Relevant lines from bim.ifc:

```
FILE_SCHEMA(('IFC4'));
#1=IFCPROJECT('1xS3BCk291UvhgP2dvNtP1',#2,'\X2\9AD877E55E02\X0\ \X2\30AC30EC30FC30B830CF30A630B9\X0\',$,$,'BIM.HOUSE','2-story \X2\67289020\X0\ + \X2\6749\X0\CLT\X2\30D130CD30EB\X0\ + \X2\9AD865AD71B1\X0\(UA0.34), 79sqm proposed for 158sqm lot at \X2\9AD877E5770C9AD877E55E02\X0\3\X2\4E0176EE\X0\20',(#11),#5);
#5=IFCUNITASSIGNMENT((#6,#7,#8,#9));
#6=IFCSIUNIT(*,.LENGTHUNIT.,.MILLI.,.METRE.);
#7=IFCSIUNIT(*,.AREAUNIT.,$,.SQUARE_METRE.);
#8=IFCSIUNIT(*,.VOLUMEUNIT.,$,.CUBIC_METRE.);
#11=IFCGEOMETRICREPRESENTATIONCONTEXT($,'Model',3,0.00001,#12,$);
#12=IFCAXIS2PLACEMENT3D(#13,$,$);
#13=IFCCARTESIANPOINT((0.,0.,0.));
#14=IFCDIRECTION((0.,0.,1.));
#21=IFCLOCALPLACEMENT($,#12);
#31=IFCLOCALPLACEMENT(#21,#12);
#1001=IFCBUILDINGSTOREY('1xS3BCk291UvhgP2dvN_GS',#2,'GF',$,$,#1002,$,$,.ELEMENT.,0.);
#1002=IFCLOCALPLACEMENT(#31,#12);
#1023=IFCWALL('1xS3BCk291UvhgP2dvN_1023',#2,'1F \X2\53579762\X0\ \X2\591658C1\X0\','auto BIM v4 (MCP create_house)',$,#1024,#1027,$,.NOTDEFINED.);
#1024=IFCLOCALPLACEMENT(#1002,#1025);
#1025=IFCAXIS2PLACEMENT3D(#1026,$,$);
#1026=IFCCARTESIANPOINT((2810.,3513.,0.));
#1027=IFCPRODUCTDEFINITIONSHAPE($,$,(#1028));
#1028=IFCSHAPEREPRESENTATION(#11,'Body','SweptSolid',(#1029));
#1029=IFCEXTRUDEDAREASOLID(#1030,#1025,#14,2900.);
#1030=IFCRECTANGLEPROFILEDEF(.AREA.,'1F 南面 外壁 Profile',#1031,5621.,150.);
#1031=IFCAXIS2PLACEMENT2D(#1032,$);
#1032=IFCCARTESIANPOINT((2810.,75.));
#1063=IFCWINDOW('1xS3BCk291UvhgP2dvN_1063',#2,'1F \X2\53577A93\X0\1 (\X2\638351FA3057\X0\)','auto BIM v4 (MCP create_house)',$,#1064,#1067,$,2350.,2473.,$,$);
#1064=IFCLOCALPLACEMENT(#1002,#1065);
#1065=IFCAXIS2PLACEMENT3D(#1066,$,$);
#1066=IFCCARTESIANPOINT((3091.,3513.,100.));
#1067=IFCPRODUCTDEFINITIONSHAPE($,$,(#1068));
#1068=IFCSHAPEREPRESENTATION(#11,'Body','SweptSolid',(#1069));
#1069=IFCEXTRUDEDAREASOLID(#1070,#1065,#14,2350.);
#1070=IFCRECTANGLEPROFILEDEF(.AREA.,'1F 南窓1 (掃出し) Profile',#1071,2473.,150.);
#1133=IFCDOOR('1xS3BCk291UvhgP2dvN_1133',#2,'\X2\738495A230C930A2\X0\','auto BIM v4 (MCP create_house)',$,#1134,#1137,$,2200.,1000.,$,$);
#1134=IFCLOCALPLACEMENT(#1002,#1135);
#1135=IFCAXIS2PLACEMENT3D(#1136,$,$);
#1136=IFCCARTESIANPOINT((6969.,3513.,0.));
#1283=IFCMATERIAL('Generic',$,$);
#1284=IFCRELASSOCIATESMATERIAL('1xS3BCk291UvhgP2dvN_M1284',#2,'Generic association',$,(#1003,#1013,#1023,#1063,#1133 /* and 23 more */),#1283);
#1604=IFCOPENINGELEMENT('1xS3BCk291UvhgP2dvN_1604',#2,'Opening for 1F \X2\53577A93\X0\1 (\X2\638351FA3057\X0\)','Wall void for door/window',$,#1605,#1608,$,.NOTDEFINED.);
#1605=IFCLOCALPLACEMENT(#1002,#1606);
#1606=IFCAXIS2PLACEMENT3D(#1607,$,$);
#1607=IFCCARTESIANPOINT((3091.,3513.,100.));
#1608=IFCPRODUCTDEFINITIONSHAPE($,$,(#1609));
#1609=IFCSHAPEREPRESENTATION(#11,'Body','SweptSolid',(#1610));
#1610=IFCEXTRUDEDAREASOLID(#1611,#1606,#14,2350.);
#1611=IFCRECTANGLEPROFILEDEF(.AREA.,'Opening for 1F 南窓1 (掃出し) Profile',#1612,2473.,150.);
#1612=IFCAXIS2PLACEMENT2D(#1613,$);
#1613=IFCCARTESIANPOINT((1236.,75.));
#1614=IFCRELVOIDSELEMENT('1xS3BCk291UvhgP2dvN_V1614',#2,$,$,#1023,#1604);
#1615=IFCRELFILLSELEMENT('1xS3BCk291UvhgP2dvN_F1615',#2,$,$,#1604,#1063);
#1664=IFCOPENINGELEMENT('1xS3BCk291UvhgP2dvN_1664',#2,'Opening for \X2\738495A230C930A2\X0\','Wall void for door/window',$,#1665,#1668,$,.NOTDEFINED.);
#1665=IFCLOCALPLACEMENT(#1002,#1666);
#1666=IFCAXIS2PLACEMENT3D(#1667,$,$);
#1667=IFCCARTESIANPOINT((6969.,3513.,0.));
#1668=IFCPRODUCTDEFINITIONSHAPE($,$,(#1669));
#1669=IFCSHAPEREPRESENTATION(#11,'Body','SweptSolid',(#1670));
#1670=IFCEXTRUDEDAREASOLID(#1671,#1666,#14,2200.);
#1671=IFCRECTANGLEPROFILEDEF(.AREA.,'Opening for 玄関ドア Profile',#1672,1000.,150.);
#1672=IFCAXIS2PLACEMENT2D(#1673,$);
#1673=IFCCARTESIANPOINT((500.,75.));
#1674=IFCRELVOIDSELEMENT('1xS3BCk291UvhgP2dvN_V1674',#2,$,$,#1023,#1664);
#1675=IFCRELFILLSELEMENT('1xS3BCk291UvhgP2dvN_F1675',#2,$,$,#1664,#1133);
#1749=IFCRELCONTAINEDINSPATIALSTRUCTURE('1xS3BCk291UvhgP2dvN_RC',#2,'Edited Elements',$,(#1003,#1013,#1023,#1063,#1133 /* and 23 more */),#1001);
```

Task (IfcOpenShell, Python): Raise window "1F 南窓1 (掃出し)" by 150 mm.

```python
import numpy as np
import ifcopenshell
import ifcopenshell.api.geometry
import ifcopenshell.util.placement
import ifcopenshell.util.unit

model = ifcopenshell.open("bim.ifc")
unit_scale = ifcopenshell.util.unit.calculate_unit_scale(model)

window = model.by_guid("1xS3BCk291UvhgP2dvN_1063")
opening = window.FillsVoids[0].RelatingOpeningElement
dz = 0.15 / unit_scale

shift = np.array([0.0, 0.0, dz])
# The window is not placed relative to its opening, so move both.
for product in (opening, window):
    matrix = ifcopenshell.util.placement.get_local_placement(product.ObjectPlacement)
    matrix[:3, 3] += shift
    ifcopenshell.api.geometry.edit_object_placement(model, product=product, matrix=matrix, is_si=False)

print(f"moved by {dz * unit_scale:+.3f} m")

model.write("bim_v2.ifc")
```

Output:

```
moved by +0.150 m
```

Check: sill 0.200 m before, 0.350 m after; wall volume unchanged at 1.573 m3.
